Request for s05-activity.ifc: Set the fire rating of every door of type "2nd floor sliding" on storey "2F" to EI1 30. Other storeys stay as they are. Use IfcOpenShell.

First a look at what the model holds.

```python
import ifcopenshell
import ifcopenshell.util.element

model = ifcopenshell.open("s05-activity.ifc")
print(model.schema)
storey = next(s for s in model.by_type("IfcBuildingStorey") if s.Name == "2F")
doors = [e for e in ifcopenshell.util.element.get_decomposition(storey) if e.is_a("IfcDoor")]
seen = {}
for e in doors:
    element_type = ifcopenshell.util.element.get_type(e)
    key = (element_type.Name if element_type != e and element_type else None, ifcopenshell.util.element.get_pset(e, "Pset_DoorCommon", "FireRating"))
    seen[key] = seen.get(key, 0) + 1
for (name, value), count in sorted(seen.items(), key=str):
    print(count, "x", name, "|", value)
```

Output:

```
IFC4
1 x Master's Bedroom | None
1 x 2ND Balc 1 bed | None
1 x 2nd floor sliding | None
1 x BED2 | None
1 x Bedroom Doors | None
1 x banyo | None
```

```python
import ifcopenshell
import ifcopenshell.api.pset
import ifcopenshell.util.element

model = ifcopenshell.open("s05-activity.ifc")

storey = next(s for s in model.by_type("IfcBuildingStorey") if s.Name == "2F")
doors = [e for e in ifcopenshell.util.element.get_decomposition(storey) if e.is_a("IfcDoor")]

count = 0
for e in doors:
    element_type = ifcopenshell.util.element.get_type(e)
    if element_type in (None, e) or element_type.Name != "2nd floor sliding":
        continue
    # add_pset returns the element's existing set when there is one.
    pset = ifcopenshell.api.pset.add_pset(model, product=e, name="Pset_DoorCommon")
    ifcopenshell.api.pset.edit_pset(model, pset=pset, properties={"FireRating": "EI1 30"})
    count += 1

print(count, "doors updated")

model.write("s05-activity_v2.ifc")
```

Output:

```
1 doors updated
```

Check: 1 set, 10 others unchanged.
